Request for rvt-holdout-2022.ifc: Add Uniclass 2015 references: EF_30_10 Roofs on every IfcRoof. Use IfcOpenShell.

First a look at what the model holds.

```python
import ifcopenshell

model = ifcopenshell.open("rvt-holdout-2022.ifc")
print(model.schema)
print("classifications:", [c.Name for c in model.by_type("IfcClassification")])
for ifc_class in ("IfcDoor", "IfcRoof", "IfcStair", "IfcWall", "IfcWindow"):
    print(ifc_class, len(model.by_type(ifc_class)))
```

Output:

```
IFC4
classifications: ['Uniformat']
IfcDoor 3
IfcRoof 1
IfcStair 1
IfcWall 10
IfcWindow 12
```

```python
import ifcopenshell
import ifcopenshell.api.classification

model = ifcopenshell.open("rvt-holdout-2022.ifc")

system = ifcopenshell.api.classification.add_classification(model, classification="Uniclass 2015")

codes = {
    "IfcRoof": ("EF_30_10", "Roofs"),
}
for ifc_class, (code, name) in codes.items():
    products = model.by_type(ifc_class)
    ifcopenshell.api.classification.add_reference(
        model, products=products, classification=system, identification=code, name=name
    )
    print(code, len(products))

model.write("rvt-holdout-2022-out.ifc")
```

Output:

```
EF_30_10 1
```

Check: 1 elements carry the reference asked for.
